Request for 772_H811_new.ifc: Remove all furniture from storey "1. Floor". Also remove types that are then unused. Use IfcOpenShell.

First a look at what the model holds.

```python
import ifcopenshell
import ifcopenshell.util.element

model = ifcopenshell.open("772_H811_new.ifc")
print(model.schema)
storey = next(s for s in model.by_type("IfcBuildingStorey") if s.Name == "1. Floor")
furniture = [e for e in ifcopenshell.util.element.get_decomposition(storey) if e.is_a("IfcFurnishingElement")]
seen = {}
for e in furniture:
    element_type = ifcopenshell.util.element.get_type(e)
    name = element_type.Name if element_type not in (None, e) else None
    seen[name] = seen.get(name, 0) + 1
for name, count in sorted(seen.items(), key=str):
    print(count, "x", name)
```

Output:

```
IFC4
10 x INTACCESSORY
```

```python
import ifcopenshell
import ifcopenshell.api.root
import ifcopenshell.util.element

model = ifcopenshell.open("772_H811_new.ifc")

storey = next(s for s in model.by_type("IfcBuildingStorey") if s.Name == "1. Floor")
furniture = [e for e in ifcopenshell.util.element.get_decomposition(storey) if e.is_a("IfcFurnishingElement")]
types = {ifcopenshell.util.element.get_type(e) for e in furniture} - {None, *furniture}

for e in furniture:
    ifcopenshell.api.root.remove_product(model, product=e)
print(len(furniture), "removed")

unused = [t for t in types if not ifcopenshell.util.element.get_types(t)]
for t in unused:
    ifcopenshell.api.root.remove_product(model, product=t)
print(len(unused), "unused types removed")

model.write("772_H811_new_rev.ifc")
```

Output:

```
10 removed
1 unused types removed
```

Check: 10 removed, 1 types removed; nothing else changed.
